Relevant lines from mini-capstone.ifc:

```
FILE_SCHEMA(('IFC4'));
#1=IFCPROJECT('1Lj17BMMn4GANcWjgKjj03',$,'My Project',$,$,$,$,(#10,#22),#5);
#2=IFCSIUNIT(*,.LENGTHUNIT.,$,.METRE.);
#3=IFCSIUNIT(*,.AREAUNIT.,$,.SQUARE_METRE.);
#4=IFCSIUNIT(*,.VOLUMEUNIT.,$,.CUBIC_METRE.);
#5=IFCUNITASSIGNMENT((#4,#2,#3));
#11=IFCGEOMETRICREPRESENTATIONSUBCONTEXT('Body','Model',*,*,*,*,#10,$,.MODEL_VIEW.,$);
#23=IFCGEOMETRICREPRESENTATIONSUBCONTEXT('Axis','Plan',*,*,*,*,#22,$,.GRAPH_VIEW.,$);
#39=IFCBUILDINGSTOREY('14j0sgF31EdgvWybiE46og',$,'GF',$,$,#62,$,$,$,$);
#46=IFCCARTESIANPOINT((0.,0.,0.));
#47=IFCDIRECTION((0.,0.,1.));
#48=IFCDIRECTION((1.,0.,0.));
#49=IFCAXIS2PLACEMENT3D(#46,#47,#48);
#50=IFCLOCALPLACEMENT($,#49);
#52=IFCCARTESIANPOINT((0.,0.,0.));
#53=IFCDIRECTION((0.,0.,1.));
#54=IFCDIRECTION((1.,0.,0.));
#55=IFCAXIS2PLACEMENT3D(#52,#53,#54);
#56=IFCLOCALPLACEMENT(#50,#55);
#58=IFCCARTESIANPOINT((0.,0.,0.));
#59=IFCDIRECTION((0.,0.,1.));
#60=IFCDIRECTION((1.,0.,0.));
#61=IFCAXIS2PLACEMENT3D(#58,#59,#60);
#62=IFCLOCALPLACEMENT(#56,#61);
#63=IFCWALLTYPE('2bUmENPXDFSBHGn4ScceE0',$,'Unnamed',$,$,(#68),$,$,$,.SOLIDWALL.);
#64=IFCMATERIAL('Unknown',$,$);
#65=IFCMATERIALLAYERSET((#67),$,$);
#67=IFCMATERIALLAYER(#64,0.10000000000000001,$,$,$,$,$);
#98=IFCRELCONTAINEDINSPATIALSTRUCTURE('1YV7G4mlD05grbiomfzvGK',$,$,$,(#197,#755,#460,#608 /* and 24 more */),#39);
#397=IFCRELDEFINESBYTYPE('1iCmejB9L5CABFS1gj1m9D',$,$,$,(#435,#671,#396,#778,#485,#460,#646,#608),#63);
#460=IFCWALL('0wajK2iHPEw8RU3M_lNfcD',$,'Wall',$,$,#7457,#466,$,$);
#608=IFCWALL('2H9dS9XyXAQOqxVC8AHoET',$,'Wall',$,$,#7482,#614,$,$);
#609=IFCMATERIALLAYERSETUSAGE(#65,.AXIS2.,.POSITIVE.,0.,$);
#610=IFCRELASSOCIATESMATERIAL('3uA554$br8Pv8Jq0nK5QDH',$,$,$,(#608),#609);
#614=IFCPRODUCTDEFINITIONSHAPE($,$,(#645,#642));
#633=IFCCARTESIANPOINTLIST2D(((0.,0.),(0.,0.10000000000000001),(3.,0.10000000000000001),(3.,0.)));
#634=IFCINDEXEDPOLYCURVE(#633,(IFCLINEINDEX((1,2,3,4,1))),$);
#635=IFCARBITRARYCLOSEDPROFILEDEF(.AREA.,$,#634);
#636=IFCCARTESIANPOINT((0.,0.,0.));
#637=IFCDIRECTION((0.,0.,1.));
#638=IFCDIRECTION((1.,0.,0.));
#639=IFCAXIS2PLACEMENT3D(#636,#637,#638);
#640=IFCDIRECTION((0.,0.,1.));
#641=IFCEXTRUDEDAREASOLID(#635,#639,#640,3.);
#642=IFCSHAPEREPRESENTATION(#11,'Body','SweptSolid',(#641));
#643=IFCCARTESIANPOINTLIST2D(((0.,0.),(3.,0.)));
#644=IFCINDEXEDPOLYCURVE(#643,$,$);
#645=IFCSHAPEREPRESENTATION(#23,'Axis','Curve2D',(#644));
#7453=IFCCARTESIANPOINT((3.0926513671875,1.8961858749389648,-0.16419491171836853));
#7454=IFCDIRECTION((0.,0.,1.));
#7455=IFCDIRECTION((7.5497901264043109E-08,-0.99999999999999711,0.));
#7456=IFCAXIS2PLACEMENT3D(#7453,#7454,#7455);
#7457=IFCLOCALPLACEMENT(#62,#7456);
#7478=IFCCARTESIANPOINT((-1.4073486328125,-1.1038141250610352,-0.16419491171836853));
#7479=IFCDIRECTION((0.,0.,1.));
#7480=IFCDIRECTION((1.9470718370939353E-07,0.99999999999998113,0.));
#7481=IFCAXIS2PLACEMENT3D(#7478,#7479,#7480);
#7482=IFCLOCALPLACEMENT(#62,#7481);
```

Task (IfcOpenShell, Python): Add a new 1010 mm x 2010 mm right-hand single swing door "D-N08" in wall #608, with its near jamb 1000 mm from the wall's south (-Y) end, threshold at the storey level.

```python
import numpy as np
import ifcopenshell
import ifcopenshell.api.feature
import ifcopenshell.api.geometry
import ifcopenshell.api.root
import ifcopenshell.api.spatial
import ifcopenshell.geom
import ifcopenshell.util.element
import ifcopenshell.util.placement
import ifcopenshell.util.representation
import ifcopenshell.util.shape
import ifcopenshell.util.unit

model = ifcopenshell.open("mini-capstone.ifc")
unit_scale = ifcopenshell.util.unit.calculate_unit_scale(model)
settings = ifcopenshell.geom.settings()


def volume(element):
    """Net volume in cubic metres, openings subtracted."""
    shape = ifcopenshell.geom.create_shape(settings, element)
    return ifcopenshell.util.shape.get_volume(shape.geometry)


wall = model.by_guid("2H9dS9XyXAQOqxVC8AHoET")
storey = ifcopenshell.util.element.get_container(wall, ifc_class="IfcBuildingStorey")
context = ifcopenshell.util.representation.get_context(model, "Model", "Body", "MODEL_VIEW")
before = volume(wall)

width, height, from_end, sill = 1.01, 2.01, 1, 0.0  # metres

# The wall runs along its own X axis, and the end named is its -X end.
wall_shape = ifcopenshell.geom.create_shape(settings, wall)
x, y, z = ifcopenshell.util.shape.get_vertices(wall_shape.geometry).T
start = x.min() + from_end
face, thickness = float(y.min()), float(y.max() - y.min())
wall_matrix = ifcopenshell.util.placement.get_local_placement(wall.ObjectPlacement)
level = ifcopenshell.util.placement.get_local_placement(storey.ObjectPlacement)[2, 3]


def in_wall(x, y):
    """Placement at x, y metres in the wall's axes, at sill height."""
    matrix = wall_matrix.copy()
    matrix[:, 3] = wall_matrix @ np.array([x / unit_scale, y / unit_scale, 0.0, 1.0])
    matrix[2, 3] = level + sill / unit_scale
    return matrix


# Opening: a box that overshoots both wall faces by 50 mm.
opening = ifcopenshell.api.root.create_entity(model, ifc_class="IfcOpeningElement", predefined_type="OPENING")
box = ifcopenshell.api.geometry.add_wall_representation(
    model, context=context, length=width, height=height, thickness=thickness + 0.1
)
ifcopenshell.api.geometry.assign_representation(model, product=opening, representation=box)
ifcopenshell.api.geometry.edit_object_placement(model, product=opening, matrix=in_wall(start, face - 0.05), is_si=False)
ifcopenshell.api.feature.add_feature(model, feature=opening, element=wall)

door = ifcopenshell.api.root.create_entity(model, ifc_class="IfcDoor", name="D-N08", predefined_type="DOOR")
door.OverallWidth, door.OverallHeight = width / unit_scale, height / unit_scale
door.OperationType = "SINGLE_SWING_RIGHT"
body = ifcopenshell.api.geometry.add_door_representation(
    model,
    context=context,
    overall_width=door.OverallWidth,
    overall_height=door.OverallHeight,
    operation_type="SINGLE_SWING_RIGHT",
    lining_properties={"LiningDepth": thickness / unit_scale, "ThresholdDepth": thickness / unit_scale},
)
ifcopenshell.api.geometry.assign_representation(model, product=door, representation=body)
ifcopenshell.api.spatial.assign_container(model, products=[door], relating_structure=storey)
ifcopenshell.api.feature.add_filling(model, opening=opening, element=door)

# The lining spans the wall, so the door starts at the wall face.
ifcopenshell.api.geometry.edit_object_placement(model, product=door, matrix=in_wall(start, face), is_si=False)

after = volume(wall)

print(f"wall volume {before:.3f} -> {after:.3f} m3")

model.write("mini-capstone_updated.ifc")
```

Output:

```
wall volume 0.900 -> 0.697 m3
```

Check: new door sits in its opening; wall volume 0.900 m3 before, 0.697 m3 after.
